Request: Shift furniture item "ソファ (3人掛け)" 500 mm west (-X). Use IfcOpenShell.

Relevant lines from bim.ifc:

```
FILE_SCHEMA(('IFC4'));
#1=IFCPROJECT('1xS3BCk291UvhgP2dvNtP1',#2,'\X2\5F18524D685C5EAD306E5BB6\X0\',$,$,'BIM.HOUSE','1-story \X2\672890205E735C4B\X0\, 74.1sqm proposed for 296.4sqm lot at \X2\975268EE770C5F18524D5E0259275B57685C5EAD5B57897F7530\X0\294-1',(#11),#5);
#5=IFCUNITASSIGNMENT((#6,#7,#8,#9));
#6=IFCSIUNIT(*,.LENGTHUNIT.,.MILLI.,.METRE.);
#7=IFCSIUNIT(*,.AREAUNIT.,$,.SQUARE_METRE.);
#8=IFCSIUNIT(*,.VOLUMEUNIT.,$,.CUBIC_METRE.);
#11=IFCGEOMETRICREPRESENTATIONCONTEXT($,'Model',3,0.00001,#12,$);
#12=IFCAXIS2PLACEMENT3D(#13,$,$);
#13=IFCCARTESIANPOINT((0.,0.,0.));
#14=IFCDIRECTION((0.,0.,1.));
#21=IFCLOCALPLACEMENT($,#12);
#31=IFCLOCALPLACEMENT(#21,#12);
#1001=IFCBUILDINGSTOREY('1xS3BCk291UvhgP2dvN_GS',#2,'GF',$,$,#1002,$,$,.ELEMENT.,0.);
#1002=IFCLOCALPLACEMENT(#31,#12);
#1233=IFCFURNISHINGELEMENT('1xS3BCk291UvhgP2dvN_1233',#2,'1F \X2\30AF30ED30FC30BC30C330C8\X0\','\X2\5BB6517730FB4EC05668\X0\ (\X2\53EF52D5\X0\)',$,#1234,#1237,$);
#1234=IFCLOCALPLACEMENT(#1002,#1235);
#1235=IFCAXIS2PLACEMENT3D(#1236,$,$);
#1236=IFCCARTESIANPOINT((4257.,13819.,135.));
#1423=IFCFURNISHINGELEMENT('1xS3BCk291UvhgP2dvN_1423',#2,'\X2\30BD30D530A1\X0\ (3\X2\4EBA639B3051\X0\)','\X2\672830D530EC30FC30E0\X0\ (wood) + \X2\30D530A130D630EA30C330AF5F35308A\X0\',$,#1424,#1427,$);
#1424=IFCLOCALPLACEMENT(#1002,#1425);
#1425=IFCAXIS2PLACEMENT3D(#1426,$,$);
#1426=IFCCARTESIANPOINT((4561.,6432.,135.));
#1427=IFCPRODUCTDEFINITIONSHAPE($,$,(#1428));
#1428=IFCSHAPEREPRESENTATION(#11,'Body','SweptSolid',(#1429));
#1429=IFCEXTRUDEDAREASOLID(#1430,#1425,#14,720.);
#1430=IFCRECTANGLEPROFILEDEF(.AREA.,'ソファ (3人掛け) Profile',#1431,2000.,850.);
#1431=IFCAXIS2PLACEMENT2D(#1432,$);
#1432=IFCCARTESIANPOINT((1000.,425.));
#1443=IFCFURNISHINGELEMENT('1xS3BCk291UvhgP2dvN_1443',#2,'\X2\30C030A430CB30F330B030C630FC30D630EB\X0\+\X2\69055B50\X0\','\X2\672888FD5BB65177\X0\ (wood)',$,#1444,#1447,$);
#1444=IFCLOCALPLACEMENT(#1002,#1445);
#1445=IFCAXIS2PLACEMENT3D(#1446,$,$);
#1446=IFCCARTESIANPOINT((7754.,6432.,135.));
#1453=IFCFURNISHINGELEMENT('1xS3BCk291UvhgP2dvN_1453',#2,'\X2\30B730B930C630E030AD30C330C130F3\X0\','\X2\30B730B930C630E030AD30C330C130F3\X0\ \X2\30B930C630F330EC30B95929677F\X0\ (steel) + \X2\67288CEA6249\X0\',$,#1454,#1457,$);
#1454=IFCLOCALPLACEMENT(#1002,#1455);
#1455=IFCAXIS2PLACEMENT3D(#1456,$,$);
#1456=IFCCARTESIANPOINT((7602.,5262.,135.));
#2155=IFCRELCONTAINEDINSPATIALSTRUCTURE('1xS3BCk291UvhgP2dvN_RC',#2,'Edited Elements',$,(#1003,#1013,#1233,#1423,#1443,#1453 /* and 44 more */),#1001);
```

```python
import ifcopenshell
import ifcopenshell.api.geometry
import ifcopenshell.util.placement

model = ifcopenshell.open("bim.ifc")

item = model.by_guid("1xS3BCk291UvhgP2dvN_1423")
matrix = ifcopenshell.util.placement.get_local_placement(item.ObjectPlacement)
matrix[0, 3] -= 500.0
ifcopenshell.api.geometry.edit_object_placement(model, product=item, matrix=matrix, is_si=False)

print(ifcopenshell.util.placement.get_local_placement(item.ObjectPlacement).round(3) + 0.0)

model.write("bim_edited.ifc")
```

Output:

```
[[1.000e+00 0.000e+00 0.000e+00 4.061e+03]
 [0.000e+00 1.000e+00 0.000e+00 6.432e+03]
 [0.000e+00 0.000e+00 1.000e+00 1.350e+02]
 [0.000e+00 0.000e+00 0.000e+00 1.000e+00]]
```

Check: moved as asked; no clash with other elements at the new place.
